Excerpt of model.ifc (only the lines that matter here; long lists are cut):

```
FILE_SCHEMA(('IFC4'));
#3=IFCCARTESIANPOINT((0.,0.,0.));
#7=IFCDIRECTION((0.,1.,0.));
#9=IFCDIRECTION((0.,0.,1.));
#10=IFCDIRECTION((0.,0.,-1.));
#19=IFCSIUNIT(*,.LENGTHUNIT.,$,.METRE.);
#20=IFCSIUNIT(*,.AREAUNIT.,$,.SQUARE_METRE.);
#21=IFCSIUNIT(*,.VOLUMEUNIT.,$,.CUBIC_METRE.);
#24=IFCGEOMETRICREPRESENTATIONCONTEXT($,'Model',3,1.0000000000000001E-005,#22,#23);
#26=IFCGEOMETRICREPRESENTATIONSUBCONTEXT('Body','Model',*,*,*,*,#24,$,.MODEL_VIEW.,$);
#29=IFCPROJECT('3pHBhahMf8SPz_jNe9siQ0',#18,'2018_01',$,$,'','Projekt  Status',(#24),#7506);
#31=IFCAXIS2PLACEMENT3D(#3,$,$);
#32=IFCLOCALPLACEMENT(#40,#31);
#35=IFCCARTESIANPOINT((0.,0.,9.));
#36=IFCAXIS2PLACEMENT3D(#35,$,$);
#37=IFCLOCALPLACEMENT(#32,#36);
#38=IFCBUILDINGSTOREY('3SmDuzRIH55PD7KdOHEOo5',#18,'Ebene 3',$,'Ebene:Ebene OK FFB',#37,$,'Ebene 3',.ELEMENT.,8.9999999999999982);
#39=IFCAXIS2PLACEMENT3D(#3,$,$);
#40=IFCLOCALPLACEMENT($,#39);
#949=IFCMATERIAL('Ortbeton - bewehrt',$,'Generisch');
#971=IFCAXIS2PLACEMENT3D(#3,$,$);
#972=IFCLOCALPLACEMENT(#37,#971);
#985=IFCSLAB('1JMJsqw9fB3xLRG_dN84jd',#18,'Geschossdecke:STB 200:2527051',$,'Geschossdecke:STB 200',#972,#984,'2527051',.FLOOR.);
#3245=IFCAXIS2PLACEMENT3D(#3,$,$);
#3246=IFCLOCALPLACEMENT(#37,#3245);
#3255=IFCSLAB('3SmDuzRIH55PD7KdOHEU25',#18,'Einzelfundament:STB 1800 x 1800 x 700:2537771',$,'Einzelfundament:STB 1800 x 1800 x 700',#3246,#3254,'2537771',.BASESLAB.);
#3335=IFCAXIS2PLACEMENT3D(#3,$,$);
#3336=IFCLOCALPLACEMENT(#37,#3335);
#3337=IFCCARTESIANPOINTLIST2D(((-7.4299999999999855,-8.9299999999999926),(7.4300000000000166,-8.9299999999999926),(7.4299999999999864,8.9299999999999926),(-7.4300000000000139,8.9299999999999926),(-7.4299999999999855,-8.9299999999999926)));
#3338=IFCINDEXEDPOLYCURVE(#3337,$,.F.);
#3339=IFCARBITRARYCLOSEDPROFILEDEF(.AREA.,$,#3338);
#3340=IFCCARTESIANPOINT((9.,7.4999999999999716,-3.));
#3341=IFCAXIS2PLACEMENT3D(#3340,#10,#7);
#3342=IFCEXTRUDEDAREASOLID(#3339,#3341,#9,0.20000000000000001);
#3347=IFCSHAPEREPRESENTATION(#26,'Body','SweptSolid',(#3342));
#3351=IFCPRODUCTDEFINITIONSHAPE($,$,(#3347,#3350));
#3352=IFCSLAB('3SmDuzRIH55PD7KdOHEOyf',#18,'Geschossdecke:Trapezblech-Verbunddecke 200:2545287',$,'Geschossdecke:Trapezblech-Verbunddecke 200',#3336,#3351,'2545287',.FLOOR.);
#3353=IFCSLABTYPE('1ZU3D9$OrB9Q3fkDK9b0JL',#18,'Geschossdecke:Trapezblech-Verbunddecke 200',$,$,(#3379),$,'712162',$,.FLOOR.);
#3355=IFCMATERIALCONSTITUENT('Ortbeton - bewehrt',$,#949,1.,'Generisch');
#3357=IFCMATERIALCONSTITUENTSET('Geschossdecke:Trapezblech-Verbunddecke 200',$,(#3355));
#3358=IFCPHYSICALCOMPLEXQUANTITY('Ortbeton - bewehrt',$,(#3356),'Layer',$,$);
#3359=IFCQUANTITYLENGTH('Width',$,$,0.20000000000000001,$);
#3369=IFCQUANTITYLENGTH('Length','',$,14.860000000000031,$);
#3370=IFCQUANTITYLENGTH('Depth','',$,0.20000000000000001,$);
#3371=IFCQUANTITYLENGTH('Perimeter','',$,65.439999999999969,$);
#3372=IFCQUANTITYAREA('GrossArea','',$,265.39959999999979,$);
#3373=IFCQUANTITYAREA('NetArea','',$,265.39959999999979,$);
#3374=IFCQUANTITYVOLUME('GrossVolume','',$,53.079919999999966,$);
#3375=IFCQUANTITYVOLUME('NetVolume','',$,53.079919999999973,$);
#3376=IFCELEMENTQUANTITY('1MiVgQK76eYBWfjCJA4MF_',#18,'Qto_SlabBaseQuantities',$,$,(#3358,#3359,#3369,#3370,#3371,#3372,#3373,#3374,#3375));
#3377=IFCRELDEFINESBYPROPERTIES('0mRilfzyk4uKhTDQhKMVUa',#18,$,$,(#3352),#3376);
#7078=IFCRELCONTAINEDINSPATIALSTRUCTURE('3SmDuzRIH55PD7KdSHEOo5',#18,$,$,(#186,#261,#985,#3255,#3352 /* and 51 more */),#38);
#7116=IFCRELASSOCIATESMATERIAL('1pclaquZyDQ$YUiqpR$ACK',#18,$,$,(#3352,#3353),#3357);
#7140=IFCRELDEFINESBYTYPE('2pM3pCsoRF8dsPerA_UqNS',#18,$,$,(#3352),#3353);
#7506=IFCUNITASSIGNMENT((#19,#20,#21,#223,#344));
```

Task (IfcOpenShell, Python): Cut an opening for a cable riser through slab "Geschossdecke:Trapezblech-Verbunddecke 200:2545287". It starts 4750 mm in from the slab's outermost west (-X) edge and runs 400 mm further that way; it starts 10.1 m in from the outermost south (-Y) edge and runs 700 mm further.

```python
import numpy as np
import ifcopenshell
import ifcopenshell.api.feature
import ifcopenshell.api.geometry
import ifcopenshell.api.pset
import ifcopenshell.api.root
import ifcopenshell.geom
import ifcopenshell.util.element
import ifcopenshell.util.placement
import ifcopenshell.util.representation
import ifcopenshell.util.shape
import ifcopenshell.util.unit

model = ifcopenshell.open("model.ifc")
unit_scale = ifcopenshell.util.unit.calculate_unit_scale(model)
area_scale = ifcopenshell.util.unit.calculate_unit_scale(model, "AREAUNIT")
volume_scale = ifcopenshell.util.unit.calculate_unit_scale(model, "VOLUMEUNIT")
settings = ifcopenshell.geom.settings()


def volume(element):
    """Net volume in cubic metres, openings subtracted."""
    shape = ifcopenshell.geom.create_shape(settings, element)
    return ifcopenshell.util.shape.get_volume(shape.geometry)


slab = model.by_id(3352)
before = volume(slab)

# Extent in the slab's own axes, in metres. The edges named are its -X and -Y sides.
slab_shape = ifcopenshell.geom.create_shape(settings, slab)
vertices = ifcopenshell.util.shape.get_vertices(slab_shape.geometry)
x_min, y_min, bottom = vertices.min(axis=0)
top = vertices[:, 2].max()

opening = ifcopenshell.api.root.create_entity(model, ifc_class="IfcOpeningElement", name="Cable riser opening", predefined_type="OPENING")
context = ifcopenshell.util.representation.get_context(model, "Model", "Body", "MODEL_VIEW")
width, depth = 0.4, 0.7
outline = [(0.0, 0.0), (width, 0.0), (width, depth), (0.0, depth), (0.0, 0.0)]
# Overshoot both faces by 50 mm so the cut is clean.
shape = ifcopenshell.api.geometry.add_slab_representation(
    model, context=context, depth=top - bottom + 0.1, polyline=outline
)
ifcopenshell.api.geometry.assign_representation(model, product=opening, representation=shape)

matrix = ifcopenshell.util.placement.get_local_placement(slab.ObjectPlacement)
matrix[:, 3] = matrix @ np.append(np.array([x_min + 4.75, y_min + 10.1, bottom - 0.05]) / unit_scale, 1.0)
ifcopenshell.api.geometry.edit_object_placement(model, product=opening, matrix=matrix, is_si=False)
ifcopenshell.api.feature.add_feature(model, feature=opening, element=slab)

after = volume(slab)

# Update the slab's stored quantities.
qto = model.by_id(ifcopenshell.util.element.get_pset(slab, "Qto_SlabBaseQuantities", should_inherit=False)["id"])
ifcopenshell.api.pset.edit_qto(model, qto=qto, properties={
    "NetArea": after / (top - bottom) / area_scale,
    "NetVolume": after / volume_scale,
})

print(f"slab volume {before:.3f} -> {after:.3f} m3")

model.write("model_updated.ifc")
```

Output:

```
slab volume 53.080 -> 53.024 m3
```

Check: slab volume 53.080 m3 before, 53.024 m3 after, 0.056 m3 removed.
